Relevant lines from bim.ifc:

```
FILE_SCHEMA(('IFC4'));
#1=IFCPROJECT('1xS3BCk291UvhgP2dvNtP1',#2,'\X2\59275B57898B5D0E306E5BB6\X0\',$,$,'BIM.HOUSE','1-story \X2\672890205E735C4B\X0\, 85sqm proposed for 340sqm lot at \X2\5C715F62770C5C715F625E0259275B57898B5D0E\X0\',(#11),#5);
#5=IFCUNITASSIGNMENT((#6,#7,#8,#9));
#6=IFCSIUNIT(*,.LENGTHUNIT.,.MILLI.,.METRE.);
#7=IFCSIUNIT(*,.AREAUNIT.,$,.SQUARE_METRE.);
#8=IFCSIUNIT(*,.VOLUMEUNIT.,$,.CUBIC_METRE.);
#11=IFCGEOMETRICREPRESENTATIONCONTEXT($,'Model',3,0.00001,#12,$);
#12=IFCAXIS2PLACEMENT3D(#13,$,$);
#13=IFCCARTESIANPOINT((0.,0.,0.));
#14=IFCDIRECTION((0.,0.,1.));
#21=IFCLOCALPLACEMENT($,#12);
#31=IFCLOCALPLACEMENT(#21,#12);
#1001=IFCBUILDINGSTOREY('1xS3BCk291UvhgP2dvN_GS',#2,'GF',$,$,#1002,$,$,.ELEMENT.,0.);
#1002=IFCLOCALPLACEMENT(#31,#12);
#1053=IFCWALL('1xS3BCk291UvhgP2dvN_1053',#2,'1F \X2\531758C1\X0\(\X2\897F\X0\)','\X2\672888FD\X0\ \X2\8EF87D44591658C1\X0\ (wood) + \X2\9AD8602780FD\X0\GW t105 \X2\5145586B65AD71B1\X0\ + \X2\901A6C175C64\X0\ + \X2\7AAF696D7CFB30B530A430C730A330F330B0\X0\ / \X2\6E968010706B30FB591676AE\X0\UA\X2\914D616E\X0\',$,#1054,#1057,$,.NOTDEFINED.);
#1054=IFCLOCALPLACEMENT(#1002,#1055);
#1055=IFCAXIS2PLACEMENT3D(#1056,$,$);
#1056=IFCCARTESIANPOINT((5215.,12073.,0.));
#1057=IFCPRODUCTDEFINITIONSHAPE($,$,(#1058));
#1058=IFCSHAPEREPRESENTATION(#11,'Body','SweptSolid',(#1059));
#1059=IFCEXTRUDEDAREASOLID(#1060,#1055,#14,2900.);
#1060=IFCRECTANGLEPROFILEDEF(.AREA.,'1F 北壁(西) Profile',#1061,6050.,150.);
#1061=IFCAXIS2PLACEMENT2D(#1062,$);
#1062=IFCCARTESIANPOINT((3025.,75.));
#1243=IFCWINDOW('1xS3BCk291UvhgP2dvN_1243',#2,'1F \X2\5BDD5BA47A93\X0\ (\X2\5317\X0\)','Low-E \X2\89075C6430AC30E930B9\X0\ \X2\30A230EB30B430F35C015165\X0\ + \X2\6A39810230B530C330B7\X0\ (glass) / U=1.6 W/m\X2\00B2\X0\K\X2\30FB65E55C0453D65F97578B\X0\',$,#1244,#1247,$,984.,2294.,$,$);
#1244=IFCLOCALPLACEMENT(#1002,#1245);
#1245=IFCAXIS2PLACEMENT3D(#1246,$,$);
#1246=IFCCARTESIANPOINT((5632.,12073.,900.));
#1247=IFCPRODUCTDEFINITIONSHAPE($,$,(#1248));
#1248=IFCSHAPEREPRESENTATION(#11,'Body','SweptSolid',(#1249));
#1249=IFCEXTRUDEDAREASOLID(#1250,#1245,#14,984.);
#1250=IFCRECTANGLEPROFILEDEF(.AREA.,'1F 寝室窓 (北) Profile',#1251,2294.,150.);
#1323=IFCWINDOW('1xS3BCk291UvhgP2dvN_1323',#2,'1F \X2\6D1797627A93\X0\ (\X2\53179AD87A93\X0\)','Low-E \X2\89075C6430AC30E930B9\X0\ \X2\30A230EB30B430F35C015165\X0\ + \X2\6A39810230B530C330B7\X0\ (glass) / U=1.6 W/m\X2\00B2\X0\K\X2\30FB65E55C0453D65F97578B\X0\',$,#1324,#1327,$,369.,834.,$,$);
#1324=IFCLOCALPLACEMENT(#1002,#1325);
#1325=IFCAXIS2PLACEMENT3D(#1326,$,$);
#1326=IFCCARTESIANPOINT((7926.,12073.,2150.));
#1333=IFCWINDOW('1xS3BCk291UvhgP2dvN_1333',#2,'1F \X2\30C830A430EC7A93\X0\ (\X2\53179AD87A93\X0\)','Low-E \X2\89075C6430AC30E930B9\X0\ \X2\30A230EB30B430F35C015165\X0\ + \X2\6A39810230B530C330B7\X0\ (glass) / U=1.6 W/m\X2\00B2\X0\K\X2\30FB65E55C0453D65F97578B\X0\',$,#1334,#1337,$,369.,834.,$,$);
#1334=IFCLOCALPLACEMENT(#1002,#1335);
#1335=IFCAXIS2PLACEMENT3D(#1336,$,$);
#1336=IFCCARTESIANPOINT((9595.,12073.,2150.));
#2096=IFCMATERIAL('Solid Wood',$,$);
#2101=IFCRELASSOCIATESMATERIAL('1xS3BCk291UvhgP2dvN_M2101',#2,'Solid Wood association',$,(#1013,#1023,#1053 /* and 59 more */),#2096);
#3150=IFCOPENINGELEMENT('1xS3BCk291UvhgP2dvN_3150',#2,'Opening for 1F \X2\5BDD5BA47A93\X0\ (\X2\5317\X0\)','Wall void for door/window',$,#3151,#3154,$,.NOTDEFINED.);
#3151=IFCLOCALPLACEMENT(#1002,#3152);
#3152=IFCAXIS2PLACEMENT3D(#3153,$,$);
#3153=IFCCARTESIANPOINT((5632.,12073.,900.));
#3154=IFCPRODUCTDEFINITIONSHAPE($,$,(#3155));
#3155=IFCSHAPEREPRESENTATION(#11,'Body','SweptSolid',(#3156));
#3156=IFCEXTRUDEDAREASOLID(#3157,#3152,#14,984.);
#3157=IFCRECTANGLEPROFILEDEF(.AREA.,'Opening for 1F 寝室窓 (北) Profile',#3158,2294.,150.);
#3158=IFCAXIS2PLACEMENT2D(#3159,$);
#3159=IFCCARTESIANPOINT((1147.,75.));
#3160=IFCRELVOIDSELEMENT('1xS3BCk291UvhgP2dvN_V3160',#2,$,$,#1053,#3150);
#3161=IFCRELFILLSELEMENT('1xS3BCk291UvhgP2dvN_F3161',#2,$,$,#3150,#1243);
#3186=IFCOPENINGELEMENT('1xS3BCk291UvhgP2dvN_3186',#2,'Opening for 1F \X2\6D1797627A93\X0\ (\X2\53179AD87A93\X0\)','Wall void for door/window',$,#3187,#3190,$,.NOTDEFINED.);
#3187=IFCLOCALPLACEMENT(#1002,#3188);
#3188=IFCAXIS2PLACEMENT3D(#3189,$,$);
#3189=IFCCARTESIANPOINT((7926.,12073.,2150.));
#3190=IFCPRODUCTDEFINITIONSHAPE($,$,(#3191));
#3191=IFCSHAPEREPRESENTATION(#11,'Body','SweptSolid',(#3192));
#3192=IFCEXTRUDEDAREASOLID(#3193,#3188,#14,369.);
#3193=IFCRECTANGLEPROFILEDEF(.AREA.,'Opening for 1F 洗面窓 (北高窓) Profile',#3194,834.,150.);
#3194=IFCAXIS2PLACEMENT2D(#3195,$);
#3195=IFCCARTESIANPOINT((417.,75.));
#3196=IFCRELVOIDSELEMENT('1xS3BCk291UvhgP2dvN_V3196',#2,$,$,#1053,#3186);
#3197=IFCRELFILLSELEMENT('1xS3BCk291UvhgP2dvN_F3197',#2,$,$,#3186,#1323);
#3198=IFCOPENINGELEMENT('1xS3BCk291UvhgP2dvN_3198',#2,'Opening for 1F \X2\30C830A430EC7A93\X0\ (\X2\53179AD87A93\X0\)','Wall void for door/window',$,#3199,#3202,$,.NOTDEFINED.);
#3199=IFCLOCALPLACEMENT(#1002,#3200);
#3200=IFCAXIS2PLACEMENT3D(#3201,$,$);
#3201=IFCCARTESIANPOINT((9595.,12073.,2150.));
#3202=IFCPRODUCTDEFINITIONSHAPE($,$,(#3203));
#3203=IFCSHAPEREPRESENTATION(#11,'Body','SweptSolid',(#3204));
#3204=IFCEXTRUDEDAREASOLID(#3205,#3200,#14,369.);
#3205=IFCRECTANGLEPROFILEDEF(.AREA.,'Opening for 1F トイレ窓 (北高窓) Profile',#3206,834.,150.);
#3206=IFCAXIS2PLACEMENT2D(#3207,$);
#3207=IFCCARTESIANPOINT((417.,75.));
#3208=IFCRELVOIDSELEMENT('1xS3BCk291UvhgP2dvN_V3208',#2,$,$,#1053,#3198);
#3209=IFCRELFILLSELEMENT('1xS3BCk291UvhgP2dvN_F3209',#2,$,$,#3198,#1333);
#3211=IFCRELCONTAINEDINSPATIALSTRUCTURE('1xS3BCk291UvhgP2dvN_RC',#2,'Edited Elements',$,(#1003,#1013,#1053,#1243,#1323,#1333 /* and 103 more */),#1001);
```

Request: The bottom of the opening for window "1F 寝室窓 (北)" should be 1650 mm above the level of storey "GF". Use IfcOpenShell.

```python
import numpy as np
import ifcopenshell
import ifcopenshell.api.geometry
import ifcopenshell.geom
import ifcopenshell.util.element
import ifcopenshell.util.placement
import ifcopenshell.util.shape
import ifcopenshell.util.unit

model = ifcopenshell.open("bim.ifc")
unit_scale = ifcopenshell.util.unit.calculate_unit_scale(model)

window = model.by_id(1243)
opening = window.FillsVoids[0].RelatingOpeningElement
storey = ifcopenshell.util.element.get_container(window, ifc_class="IfcBuildingStorey")
level = ifcopenshell.util.placement.get_local_placement(storey.ObjectPlacement)[2, 3]

# The opening's origin need not be at the sill, so measure its lowest point.
shape = ifcopenshell.geom.create_shape(ifcopenshell.geom.settings(), opening)
bottom = ifcopenshell.util.shape.get_shape_bottom_elevation(shape, shape.geometry) / unit_scale
dz = level + 1.65 / unit_scale - bottom

shift = np.array([0.0, 0.0, dz])
# The window is not placed relative to its opening, so move both.
for product in (opening, window):
    matrix = ifcopenshell.util.placement.get_local_placement(product.ObjectPlacement)
    matrix[:3, 3] += shift
    ifcopenshell.api.geometry.edit_object_placement(model, product=product, matrix=matrix, is_si=False)

print(f"moved by {dz * unit_scale:+.3f} m")

model.write("bim-out.ifc")
```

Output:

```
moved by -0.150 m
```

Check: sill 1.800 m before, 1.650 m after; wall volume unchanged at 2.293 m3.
